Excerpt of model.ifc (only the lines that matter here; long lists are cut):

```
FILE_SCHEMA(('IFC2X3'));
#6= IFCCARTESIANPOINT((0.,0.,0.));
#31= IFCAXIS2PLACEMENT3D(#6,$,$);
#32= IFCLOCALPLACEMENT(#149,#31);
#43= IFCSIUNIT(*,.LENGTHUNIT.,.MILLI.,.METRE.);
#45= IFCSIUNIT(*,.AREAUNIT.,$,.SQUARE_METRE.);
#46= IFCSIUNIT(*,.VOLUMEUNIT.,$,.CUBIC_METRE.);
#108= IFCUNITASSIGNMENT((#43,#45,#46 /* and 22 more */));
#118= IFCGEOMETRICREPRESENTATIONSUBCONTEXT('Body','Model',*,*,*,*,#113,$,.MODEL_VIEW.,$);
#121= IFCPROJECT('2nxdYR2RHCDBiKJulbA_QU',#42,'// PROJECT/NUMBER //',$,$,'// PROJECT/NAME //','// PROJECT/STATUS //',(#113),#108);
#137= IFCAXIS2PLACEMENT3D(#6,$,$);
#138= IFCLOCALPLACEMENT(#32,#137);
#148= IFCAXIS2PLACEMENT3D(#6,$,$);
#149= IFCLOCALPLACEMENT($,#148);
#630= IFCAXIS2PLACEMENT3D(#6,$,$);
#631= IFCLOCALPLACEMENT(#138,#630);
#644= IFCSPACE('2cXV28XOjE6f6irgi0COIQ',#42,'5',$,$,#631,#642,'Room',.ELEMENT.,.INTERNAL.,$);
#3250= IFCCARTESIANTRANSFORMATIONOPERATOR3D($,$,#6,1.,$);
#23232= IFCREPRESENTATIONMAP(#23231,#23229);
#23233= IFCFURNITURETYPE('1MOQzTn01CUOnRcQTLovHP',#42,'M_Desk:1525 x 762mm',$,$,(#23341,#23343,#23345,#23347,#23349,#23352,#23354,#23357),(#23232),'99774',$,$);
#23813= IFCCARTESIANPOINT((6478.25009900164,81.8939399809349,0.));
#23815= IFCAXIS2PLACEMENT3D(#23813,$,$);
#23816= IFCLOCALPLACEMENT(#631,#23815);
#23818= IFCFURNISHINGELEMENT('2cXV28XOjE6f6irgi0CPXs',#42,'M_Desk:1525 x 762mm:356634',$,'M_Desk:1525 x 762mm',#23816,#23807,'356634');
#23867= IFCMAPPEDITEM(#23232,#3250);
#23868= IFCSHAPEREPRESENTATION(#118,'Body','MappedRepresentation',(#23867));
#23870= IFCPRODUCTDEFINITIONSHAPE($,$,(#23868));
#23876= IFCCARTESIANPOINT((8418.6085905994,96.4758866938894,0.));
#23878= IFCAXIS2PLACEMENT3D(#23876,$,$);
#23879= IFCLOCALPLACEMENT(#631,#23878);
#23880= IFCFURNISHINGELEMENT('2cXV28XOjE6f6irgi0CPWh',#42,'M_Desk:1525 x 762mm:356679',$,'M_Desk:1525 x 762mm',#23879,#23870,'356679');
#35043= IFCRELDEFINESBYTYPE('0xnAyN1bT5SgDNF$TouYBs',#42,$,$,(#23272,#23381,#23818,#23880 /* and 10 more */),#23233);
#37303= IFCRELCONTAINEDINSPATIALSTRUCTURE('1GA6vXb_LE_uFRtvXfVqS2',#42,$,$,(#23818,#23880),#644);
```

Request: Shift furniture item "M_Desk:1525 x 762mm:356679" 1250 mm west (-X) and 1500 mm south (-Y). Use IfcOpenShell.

```python
import ifcopenshell
import ifcopenshell.api.geometry
import ifcopenshell.util.placement

model = ifcopenshell.open("model.ifc")

item = model.by_guid("2cXV28XOjE6f6irgi0CPWh")
matrix = ifcopenshell.util.placement.get_local_placement(item.ObjectPlacement)
matrix[0, 3] -= 1250.0
matrix[1, 3] -= 1500.0
ifcopenshell.api.geometry.edit_object_placement(model, product=item, matrix=matrix, is_si=False)

print(ifcopenshell.util.placement.get_local_placement(item.ObjectPlacement).round(3) + 0.0)

model.write("model_v2.ifc")
```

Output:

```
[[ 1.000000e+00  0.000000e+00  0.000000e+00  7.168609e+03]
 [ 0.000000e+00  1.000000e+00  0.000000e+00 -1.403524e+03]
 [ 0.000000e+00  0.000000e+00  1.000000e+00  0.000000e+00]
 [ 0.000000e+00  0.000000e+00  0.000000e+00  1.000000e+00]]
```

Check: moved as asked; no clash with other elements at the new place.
